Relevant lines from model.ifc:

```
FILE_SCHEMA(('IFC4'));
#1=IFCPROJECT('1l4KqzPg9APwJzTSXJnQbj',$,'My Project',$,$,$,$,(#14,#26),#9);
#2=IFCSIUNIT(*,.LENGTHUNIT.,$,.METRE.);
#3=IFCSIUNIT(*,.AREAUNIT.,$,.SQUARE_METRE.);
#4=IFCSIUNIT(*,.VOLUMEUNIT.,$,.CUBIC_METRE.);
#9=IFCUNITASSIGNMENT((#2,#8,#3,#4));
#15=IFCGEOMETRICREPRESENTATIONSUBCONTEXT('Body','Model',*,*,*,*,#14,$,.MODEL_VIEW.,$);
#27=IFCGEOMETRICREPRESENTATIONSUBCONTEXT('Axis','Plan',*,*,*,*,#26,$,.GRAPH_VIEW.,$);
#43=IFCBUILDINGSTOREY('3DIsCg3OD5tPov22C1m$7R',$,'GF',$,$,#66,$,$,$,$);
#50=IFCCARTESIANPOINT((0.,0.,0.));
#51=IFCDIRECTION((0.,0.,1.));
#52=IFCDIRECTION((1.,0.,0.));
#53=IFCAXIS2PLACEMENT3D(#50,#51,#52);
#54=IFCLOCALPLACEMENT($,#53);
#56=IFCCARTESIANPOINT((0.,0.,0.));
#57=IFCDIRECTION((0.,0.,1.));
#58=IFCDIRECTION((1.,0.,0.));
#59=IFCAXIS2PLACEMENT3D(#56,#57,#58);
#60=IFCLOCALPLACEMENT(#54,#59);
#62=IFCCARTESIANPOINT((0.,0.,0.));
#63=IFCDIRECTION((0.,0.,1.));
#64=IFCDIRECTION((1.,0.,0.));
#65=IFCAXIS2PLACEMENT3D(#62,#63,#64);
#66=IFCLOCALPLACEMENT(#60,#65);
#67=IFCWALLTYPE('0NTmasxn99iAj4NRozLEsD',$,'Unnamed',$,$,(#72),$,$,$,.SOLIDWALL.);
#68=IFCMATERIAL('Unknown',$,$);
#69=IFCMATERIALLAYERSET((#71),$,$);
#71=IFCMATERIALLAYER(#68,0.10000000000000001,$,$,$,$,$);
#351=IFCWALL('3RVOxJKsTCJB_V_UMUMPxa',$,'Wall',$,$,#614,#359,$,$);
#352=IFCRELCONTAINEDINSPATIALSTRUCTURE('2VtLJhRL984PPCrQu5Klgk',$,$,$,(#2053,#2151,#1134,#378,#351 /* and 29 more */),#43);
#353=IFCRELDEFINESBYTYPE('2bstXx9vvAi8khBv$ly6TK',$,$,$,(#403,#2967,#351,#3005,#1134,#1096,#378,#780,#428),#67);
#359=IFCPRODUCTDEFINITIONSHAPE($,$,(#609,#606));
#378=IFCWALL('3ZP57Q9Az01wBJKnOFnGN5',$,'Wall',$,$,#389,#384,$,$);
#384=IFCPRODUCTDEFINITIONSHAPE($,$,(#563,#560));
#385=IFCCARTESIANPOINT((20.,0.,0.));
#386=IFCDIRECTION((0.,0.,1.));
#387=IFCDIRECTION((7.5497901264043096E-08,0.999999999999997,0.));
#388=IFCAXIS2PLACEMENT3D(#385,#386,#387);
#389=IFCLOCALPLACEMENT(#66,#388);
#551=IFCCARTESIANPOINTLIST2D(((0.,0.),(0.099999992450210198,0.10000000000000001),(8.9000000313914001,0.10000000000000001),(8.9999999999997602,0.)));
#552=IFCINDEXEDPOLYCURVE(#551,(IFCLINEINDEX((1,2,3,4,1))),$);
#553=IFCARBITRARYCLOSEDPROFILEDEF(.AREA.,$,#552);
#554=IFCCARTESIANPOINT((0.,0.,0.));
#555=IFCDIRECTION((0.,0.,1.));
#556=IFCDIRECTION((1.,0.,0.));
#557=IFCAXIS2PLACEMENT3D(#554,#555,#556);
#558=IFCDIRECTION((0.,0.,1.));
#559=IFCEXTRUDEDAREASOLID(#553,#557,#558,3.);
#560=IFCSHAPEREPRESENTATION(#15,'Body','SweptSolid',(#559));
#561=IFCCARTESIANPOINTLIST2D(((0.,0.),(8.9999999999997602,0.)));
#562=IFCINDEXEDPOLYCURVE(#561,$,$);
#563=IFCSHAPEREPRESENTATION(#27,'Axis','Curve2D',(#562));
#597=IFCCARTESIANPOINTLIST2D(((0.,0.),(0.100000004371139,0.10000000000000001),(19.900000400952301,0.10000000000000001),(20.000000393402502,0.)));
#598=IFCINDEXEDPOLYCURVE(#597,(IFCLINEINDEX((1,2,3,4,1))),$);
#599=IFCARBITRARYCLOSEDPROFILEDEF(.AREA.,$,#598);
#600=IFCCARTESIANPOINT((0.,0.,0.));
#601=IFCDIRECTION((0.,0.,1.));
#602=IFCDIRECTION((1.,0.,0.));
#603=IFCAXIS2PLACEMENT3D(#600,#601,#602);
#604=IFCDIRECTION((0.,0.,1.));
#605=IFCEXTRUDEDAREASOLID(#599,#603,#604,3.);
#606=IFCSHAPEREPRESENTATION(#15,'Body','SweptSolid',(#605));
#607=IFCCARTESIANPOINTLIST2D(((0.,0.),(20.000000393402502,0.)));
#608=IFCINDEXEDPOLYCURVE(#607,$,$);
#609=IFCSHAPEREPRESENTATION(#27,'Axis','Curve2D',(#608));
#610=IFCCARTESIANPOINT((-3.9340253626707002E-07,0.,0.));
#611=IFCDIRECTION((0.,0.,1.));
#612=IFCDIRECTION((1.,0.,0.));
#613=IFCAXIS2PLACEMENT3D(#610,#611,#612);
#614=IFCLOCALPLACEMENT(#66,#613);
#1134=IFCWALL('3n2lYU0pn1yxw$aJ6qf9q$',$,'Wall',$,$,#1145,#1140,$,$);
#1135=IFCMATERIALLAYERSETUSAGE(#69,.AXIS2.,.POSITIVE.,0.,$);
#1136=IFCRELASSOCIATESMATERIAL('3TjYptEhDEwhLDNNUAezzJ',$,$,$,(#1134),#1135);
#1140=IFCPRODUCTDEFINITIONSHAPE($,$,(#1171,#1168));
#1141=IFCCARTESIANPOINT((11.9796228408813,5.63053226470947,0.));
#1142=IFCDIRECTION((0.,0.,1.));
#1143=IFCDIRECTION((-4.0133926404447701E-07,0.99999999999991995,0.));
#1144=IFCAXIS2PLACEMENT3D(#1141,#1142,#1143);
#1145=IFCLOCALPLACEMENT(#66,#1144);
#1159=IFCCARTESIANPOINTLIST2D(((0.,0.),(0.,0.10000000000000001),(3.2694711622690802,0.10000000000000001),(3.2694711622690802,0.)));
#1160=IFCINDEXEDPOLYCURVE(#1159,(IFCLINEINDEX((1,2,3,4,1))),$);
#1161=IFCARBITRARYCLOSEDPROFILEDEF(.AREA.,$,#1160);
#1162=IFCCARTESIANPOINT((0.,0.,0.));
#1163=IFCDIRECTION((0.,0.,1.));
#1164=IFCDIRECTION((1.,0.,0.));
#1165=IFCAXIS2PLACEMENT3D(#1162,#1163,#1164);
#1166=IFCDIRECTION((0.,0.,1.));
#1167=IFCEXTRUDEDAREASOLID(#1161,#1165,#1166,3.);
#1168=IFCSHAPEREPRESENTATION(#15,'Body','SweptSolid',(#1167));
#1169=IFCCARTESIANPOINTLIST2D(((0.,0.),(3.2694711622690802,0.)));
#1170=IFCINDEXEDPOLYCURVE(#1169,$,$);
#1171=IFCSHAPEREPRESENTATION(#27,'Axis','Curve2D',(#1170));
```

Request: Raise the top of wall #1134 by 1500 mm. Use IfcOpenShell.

```python
import ifcopenshell
import ifcopenshell.geom
import ifcopenshell.util.representation
import ifcopenshell.util.shape
import ifcopenshell.util.unit

model = ifcopenshell.open("model.ifc")
unit_scale = ifcopenshell.util.unit.calculate_unit_scale(model)
settings = ifcopenshell.geom.settings()


def volume(element):
    """Net volume in cubic metres, openings subtracted."""
    shape = ifcopenshell.geom.create_shape(settings, element)
    return ifcopenshell.util.shape.get_volume(shape.geometry)


wall = model.by_guid("3n2lYU0pn1yxw$aJ6qf9q$")
before = volume(wall)

body = ifcopenshell.util.representation.get_representation(wall, "Model", "Body")
solid = body.Items[0]
old_height = solid.Depth
solid.Depth += 1.5 / unit_scale
after = volume(wall)

print(f"height {old_height:g} -> {solid.Depth:g}, volume {before:.3f} -> {after:.3f} m3")

model.write("model-out.ifc")
```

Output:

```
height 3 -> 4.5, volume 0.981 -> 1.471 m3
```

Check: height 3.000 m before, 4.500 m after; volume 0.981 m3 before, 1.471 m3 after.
